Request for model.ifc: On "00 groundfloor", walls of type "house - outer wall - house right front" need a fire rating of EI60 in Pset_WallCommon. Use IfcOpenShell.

First a look at what the model holds.

```python
import ifcopenshell
import ifcopenshell.util.element

model = ifcopenshell.open("model.ifc")
print(model.schema)
storey = next(s for s in model.by_type("IfcBuildingStorey") if s.Name == "00 groundfloor")
walls = [e for e in ifcopenshell.util.element.get_decomposition(storey) if e.is_a("IfcWall")]
seen = {}
for e in walls:
    element_type = ifcopenshell.util.element.get_type(e)
    key = (element_type.Name if element_type != e and element_type else None, ifcopenshell.util.element.get_pset(e, "Pset_WallCommon", "FireRating"))
    seen[key] = seen.get(key, 0) + 1
for (name, value), count in sorted(seen.items(), key=str):
    print(count, "x", name, "|", value)
```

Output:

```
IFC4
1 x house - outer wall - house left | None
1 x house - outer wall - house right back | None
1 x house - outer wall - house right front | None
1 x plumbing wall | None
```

```python
import ifcopenshell
import ifcopenshell.api.pset
import ifcopenshell.util.element

model = ifcopenshell.open("model.ifc")

storey = next(s for s in model.by_type("IfcBuildingStorey") if s.Name == "00 groundfloor")
walls = [e for e in ifcopenshell.util.element.get_decomposition(storey) if e.is_a("IfcWall")]

count = 0
for e in walls:
    element_type = ifcopenshell.util.element.get_type(e)
    if element_type in (None, e) or element_type.Name != "house - outer wall - house right front":
        continue
    # add_pset returns the element's existing set when there is one.
    pset = ifcopenshell.api.pset.add_pset(model, product=e, name="Pset_WallCommon")
    ifcopenshell.api.pset.edit_pset(model, pset=pset, properties={"FireRating": "EI60"})
    count += 1

print(count, "walls updated")

model.write("model_rev.ifc")
```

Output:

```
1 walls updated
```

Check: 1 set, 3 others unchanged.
